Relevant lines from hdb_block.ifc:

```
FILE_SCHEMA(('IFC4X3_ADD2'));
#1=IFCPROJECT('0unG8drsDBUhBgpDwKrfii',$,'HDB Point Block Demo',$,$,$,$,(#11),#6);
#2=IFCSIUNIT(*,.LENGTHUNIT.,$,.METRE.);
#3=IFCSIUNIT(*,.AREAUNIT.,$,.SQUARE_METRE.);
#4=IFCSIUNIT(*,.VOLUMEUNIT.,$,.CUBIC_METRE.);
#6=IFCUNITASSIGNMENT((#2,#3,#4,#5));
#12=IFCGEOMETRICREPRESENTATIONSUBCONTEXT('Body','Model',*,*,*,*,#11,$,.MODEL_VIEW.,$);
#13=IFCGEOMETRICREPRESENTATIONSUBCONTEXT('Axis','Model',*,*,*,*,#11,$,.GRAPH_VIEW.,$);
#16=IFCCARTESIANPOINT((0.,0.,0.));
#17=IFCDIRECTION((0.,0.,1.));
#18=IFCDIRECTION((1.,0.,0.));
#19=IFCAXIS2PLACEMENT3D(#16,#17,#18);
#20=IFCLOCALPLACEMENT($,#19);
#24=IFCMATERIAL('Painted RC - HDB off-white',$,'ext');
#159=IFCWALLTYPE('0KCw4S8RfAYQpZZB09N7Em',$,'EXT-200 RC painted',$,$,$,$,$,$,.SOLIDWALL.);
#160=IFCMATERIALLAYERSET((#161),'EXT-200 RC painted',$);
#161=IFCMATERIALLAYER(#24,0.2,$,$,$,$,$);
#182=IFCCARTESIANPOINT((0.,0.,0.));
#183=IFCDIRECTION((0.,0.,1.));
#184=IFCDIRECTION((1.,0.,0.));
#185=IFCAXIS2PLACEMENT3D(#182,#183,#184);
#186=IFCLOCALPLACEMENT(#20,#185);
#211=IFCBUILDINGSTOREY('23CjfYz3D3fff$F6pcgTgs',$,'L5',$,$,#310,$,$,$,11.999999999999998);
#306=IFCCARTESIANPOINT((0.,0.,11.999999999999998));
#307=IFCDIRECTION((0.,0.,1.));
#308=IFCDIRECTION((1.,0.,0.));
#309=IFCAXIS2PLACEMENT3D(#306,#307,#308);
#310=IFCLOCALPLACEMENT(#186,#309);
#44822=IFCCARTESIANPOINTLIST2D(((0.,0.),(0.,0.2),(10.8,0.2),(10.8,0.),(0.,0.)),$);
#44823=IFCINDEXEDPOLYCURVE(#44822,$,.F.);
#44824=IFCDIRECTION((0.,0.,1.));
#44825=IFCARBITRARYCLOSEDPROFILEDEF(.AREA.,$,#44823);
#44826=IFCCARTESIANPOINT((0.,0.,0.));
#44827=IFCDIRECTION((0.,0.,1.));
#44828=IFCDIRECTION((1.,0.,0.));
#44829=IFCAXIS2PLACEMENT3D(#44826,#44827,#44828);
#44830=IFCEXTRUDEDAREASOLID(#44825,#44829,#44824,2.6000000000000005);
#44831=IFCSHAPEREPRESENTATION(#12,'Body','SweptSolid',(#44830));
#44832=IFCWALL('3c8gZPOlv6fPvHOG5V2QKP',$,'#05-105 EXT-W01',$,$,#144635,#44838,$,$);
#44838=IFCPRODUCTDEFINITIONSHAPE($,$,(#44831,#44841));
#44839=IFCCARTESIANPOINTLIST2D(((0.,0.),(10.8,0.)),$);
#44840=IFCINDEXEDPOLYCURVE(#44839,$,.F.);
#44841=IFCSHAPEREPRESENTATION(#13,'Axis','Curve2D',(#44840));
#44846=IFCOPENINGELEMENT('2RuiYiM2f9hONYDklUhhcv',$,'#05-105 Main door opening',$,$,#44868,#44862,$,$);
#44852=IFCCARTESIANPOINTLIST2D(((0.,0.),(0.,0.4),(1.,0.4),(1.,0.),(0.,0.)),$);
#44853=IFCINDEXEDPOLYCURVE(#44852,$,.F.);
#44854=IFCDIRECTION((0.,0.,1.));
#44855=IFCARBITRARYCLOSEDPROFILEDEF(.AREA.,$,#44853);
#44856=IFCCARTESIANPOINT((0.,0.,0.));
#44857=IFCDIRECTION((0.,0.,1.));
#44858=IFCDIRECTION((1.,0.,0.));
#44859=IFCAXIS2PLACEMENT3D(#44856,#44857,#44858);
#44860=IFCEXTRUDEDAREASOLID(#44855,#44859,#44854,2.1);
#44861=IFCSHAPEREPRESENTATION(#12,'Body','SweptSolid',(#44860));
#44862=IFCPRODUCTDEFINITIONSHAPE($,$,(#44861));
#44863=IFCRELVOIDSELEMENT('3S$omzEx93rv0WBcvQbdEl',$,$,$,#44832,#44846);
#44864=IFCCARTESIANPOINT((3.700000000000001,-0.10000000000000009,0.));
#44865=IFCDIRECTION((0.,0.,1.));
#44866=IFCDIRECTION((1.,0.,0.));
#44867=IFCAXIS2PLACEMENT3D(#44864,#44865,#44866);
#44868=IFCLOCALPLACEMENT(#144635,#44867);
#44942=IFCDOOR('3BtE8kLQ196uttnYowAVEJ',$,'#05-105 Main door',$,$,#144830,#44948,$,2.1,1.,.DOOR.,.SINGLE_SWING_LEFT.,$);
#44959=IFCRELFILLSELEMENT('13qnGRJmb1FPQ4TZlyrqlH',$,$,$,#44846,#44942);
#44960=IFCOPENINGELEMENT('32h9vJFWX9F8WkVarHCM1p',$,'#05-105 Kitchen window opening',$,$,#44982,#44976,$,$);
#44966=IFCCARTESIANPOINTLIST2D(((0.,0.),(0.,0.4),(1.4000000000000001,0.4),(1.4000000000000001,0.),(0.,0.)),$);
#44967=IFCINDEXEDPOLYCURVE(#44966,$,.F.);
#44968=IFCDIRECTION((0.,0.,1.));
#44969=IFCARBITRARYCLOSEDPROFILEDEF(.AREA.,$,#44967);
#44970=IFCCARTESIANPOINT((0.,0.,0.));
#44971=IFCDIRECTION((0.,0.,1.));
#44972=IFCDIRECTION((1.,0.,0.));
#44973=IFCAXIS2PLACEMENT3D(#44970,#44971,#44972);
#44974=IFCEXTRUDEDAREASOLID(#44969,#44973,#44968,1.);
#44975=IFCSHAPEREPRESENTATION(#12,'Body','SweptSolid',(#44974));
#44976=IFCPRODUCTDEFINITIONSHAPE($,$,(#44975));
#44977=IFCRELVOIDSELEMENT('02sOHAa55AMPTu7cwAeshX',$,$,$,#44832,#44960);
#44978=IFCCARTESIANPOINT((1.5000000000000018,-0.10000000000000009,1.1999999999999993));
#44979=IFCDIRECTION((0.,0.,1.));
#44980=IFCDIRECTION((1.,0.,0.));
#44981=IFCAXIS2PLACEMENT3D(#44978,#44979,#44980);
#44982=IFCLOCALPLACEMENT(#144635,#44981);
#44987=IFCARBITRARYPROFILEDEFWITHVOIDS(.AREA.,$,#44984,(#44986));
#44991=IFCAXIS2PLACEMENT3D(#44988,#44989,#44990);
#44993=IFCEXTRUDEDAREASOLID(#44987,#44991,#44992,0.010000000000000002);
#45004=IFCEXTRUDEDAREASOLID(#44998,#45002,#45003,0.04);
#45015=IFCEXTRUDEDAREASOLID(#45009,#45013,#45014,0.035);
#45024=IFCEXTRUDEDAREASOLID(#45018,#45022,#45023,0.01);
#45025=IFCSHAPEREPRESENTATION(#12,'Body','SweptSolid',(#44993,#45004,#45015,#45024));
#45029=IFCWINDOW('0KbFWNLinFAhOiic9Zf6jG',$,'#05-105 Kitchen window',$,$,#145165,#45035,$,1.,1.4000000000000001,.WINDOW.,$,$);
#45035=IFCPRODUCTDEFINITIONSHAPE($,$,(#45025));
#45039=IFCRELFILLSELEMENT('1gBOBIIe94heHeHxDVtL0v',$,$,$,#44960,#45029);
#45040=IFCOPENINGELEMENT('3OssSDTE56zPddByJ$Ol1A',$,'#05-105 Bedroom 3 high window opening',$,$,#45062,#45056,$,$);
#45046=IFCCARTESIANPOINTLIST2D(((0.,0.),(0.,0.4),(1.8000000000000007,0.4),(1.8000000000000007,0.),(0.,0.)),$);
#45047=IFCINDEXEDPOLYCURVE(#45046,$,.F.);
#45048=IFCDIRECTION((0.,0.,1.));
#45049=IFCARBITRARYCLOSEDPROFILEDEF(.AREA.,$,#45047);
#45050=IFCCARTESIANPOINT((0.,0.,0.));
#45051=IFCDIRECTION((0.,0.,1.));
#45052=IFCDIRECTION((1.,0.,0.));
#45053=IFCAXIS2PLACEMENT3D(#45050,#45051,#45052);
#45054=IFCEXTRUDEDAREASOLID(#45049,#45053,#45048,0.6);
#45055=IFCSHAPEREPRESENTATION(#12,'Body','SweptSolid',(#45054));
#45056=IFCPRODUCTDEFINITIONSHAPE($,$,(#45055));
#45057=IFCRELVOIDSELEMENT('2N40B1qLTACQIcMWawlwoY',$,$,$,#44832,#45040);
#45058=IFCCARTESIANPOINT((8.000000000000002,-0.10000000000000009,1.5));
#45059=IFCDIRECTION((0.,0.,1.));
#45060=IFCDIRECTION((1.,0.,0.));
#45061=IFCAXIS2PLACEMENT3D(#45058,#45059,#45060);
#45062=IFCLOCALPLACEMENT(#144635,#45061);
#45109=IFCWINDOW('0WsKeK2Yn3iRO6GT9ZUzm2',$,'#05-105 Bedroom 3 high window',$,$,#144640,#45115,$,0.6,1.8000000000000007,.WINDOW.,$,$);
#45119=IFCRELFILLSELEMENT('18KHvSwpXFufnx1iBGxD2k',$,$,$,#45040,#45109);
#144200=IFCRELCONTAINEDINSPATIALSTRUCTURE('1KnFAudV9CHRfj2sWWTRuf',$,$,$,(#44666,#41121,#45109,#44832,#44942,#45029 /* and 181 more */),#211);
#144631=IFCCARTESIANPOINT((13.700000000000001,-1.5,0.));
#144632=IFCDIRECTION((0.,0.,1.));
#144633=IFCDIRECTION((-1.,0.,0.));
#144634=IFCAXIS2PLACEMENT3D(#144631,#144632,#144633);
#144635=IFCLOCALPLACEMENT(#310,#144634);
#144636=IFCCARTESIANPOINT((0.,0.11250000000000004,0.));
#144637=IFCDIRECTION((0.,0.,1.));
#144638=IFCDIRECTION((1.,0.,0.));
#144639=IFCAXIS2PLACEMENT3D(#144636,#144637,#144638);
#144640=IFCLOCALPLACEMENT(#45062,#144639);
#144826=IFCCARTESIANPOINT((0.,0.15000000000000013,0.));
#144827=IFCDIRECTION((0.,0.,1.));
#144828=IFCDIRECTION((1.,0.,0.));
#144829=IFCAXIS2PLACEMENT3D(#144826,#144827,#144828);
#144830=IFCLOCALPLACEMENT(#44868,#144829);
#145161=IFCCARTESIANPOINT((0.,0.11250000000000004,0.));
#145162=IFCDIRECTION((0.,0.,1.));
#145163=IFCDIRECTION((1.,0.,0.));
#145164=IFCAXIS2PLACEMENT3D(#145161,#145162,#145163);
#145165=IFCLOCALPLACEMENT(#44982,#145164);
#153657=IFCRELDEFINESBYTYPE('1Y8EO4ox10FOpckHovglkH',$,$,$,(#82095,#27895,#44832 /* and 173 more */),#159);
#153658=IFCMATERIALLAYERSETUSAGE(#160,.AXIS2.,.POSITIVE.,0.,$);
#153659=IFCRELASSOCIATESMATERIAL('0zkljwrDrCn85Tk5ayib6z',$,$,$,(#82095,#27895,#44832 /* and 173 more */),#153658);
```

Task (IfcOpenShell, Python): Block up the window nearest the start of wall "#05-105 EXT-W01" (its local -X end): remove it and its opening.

```python
import ifcopenshell
import ifcopenshell.api.feature
import ifcopenshell.api.root
import ifcopenshell.geom
import ifcopenshell.util.shape

model = ifcopenshell.open("hdb_block.ifc")
settings = ifcopenshell.geom.settings()


def volume(element):
    """Net volume in cubic metres, openings subtracted."""
    shape = ifcopenshell.geom.create_shape(settings, element)
    return ifcopenshell.util.shape.get_volume(shape.geometry)


window = model.by_guid("0KbFWNLinFAhOiic9Zf6jG")
opening = window.FillsVoids[0].RelatingOpeningElement
wall = opening.VoidsElements[0].RelatingBuildingElement
before = volume(wall)

ifcopenshell.api.root.remove_product(model, product=window)
ifcopenshell.api.feature.remove_feature(model, feature=opening)

after = volume(wall)

print(f"wall volume {before:.3f} -> {after:.3f} m3")

model.write("hdb_block_edited.ifc")
```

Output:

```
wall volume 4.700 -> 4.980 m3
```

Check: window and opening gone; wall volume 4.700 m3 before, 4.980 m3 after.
